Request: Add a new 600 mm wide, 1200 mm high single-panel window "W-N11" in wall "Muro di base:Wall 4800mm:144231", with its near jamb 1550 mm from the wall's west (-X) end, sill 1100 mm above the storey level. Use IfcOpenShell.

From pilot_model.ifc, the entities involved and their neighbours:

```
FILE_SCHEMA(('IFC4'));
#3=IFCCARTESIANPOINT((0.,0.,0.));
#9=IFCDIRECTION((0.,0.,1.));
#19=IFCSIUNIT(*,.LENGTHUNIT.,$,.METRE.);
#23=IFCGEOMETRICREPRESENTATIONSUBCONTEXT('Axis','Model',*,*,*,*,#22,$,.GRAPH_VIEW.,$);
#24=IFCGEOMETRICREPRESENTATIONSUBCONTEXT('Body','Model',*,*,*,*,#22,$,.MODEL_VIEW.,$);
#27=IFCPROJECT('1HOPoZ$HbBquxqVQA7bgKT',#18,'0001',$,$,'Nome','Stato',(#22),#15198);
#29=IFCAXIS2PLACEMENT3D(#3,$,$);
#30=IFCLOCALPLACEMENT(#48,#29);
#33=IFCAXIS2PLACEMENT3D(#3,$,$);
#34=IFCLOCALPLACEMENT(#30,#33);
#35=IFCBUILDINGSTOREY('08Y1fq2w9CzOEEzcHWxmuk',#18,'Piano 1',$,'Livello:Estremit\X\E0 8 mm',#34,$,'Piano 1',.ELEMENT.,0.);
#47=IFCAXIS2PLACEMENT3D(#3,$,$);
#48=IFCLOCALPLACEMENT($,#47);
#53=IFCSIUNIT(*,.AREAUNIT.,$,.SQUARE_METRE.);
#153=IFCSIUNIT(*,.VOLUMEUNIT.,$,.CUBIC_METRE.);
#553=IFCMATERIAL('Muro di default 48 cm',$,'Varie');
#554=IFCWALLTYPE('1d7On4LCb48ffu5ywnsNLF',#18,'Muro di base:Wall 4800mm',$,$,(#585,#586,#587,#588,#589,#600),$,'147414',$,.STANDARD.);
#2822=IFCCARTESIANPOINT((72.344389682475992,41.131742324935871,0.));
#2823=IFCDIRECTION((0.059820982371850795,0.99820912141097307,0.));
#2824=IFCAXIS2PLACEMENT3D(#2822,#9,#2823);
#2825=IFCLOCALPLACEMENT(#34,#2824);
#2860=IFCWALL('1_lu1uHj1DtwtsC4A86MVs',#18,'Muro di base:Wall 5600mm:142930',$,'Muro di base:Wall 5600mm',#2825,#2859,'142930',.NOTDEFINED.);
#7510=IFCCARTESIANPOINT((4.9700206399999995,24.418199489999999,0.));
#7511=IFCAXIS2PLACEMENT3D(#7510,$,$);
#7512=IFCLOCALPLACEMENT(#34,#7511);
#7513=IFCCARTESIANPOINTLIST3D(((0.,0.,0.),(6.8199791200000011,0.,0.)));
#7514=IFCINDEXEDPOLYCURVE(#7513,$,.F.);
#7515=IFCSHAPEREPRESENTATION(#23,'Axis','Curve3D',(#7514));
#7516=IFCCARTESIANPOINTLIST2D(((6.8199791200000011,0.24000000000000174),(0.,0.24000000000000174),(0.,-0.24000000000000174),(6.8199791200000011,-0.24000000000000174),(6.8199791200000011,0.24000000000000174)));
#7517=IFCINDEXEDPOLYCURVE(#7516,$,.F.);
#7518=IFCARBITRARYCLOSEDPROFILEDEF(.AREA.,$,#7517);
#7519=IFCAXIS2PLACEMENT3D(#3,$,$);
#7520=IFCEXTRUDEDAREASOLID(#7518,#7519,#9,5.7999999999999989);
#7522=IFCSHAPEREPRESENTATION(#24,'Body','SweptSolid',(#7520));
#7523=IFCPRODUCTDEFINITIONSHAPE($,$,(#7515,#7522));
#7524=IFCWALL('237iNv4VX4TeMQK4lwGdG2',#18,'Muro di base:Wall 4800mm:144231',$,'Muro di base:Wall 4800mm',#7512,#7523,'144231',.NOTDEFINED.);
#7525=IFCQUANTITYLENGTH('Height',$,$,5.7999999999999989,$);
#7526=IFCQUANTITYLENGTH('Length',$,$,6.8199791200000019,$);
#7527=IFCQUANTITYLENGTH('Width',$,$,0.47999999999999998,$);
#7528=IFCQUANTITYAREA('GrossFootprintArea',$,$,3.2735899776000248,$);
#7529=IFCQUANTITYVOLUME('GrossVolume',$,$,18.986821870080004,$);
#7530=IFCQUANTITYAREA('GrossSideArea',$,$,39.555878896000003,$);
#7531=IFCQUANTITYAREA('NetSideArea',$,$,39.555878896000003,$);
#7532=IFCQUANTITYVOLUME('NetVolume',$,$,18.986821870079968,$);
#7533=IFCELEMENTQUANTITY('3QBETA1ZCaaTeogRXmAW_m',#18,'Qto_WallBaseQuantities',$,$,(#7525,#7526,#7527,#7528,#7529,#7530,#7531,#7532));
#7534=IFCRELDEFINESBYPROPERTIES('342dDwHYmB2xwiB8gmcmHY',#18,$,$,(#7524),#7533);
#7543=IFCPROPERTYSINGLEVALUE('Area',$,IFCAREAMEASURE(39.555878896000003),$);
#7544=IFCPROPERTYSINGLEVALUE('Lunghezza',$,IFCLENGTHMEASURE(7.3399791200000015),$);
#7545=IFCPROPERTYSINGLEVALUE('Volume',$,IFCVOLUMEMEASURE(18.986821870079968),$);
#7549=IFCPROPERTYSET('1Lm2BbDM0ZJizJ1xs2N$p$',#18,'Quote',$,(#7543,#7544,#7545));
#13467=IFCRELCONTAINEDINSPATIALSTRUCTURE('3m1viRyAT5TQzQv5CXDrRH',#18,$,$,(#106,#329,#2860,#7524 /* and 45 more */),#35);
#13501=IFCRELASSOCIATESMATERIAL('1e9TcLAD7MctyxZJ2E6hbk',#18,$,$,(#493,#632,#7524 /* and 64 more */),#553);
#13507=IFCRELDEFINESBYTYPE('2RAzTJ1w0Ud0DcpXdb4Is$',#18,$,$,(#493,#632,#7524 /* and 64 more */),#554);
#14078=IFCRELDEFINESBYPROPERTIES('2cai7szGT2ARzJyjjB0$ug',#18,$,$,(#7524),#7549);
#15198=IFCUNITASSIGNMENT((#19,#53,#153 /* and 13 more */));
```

```python
import numpy as np
import ifcopenshell
import ifcopenshell.api.feature
import ifcopenshell.api.geometry
import ifcopenshell.api.pset
import ifcopenshell.api.root
import ifcopenshell.api.spatial
import ifcopenshell.geom
import ifcopenshell.util.element
import ifcopenshell.util.placement
import ifcopenshell.util.representation
import ifcopenshell.util.shape
import ifcopenshell.util.unit

model = ifcopenshell.open("pilot_model.ifc")
unit_scale = ifcopenshell.util.unit.calculate_unit_scale(model)
area_scale = ifcopenshell.util.unit.calculate_unit_scale(model, "AREAUNIT")
volume_scale = ifcopenshell.util.unit.calculate_unit_scale(model, "VOLUMEUNIT")
settings = ifcopenshell.geom.settings()


def volume(element):
    """Net volume in cubic metres, openings subtracted."""
    shape = ifcopenshell.geom.create_shape(settings, element)
    return ifcopenshell.util.shape.get_volume(shape.geometry)


wall = model.by_guid("237iNv4VX4TeMQK4lwGdG2")
storey = ifcopenshell.util.element.get_container(wall, ifc_class="IfcBuildingStorey")
context = ifcopenshell.util.representation.get_context(model, "Model", "Body", "MODEL_VIEW")
before = volume(wall)

width, height, from_end, sill = 0.6, 1.2, 1.55, 1.1  # metres

# The wall runs along its own X axis, and the end named is its -X end.
wall_shape = ifcopenshell.geom.create_shape(settings, wall)
x, y, z = ifcopenshell.util.shape.get_vertices(wall_shape.geometry).T
start = x.min() + from_end
face, thickness = float(y.min()), float(y.max() - y.min())
wall_matrix = ifcopenshell.util.placement.get_local_placement(wall.ObjectPlacement)
level = ifcopenshell.util.placement.get_local_placement(storey.ObjectPlacement)[2, 3]


def in_wall(x, y):
    """Placement at x, y metres in the wall's axes, at sill height."""
    matrix = wall_matrix.copy()
    matrix[:, 3] = wall_matrix @ np.array([x / unit_scale, y / unit_scale, 0.0, 1.0])
    matrix[2, 3] = level + sill / unit_scale
    return matrix


# Opening: a box that overshoots both wall faces by 50 mm.
opening = ifcopenshell.api.root.create_entity(model, ifc_class="IfcOpeningElement", predefined_type="OPENING")
box = ifcopenshell.api.geometry.add_wall_representation(
    model, context=context, length=width, height=height, thickness=thickness + 0.1
)
ifcopenshell.api.geometry.assign_representation(model, product=opening, representation=box)
ifcopenshell.api.geometry.edit_object_placement(model, product=opening, matrix=in_wall(start, face - 0.05), is_si=False)
ifcopenshell.api.feature.add_feature(model, feature=opening, element=wall)

window = ifcopenshell.api.root.create_entity(model, ifc_class="IfcWindow", name="W-N11", predefined_type="WINDOW")
window.OverallWidth, window.OverallHeight = width / unit_scale, height / unit_scale
window.PartitioningType = "SINGLE_PANEL"
body = ifcopenshell.api.geometry.add_window_representation(
    model,
    context=context,
    overall_width=window.OverallWidth,
    overall_height=window.OverallHeight,
    partition_type="SINGLE_PANEL",
)
ifcopenshell.api.geometry.assign_representation(model, product=window, representation=body)
ifcopenshell.api.spatial.assign_container(model, products=[window], relating_structure=storey)
ifcopenshell.api.feature.add_filling(model, opening=opening, element=window)

# Centre the window in the wall's thickness.
ifcopenshell.api.geometry.edit_object_placement(model, product=window, matrix=in_wall(start, face), is_si=False)
window_shape = ifcopenshell.geom.create_shape(settings, window)
depth = ifcopenshell.util.shape.get_vertices(window_shape.geometry)[:, 1]
offset = face + thickness / 2 - (depth.min() + depth.max()) / 2
ifcopenshell.api.geometry.edit_object_placement(model, product=window, matrix=in_wall(start, offset), is_si=False)

after = volume(wall)

# Update the wall's stored quantities.
qto = model.by_id(ifcopenshell.util.element.get_pset(wall, "Qto_WallBaseQuantities", should_inherit=False)["id"])
ifcopenshell.api.pset.edit_qto(model, qto=qto, properties={
    "NetSideArea": after / thickness / area_scale,
    "NetVolume": after / volume_scale,
})
pset = model.by_id(ifcopenshell.util.element.get_pset(wall, "Quote", should_inherit=False)["id"])
ifcopenshell.api.pset.edit_pset(model, pset=pset, properties={
    "Area": model.create_entity("IfcAreaMeasure", after / thickness / area_scale),
    "Volume": model.create_entity("IfcVolumeMeasure", after / volume_scale),
})

print(f"wall volume {before:.3f} -> {after:.3f} m3")

model.write("pilot_model_rev.ifc")
```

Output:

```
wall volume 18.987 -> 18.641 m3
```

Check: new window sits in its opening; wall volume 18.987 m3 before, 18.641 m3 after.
